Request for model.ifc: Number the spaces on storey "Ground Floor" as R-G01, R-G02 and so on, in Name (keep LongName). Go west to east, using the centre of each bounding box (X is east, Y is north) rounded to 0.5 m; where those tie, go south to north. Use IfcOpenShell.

First a look at what the model holds.

```python
import ifcopenshell
import ifcopenshell.util.element
import ifcopenshell.util.placement

model = ifcopenshell.open("model.ifc")
print(model.schema)
storey = next(s for s in model.by_type("IfcBuildingStorey") if s.Name == "Ground Floor")
spaces = [e for e in ifcopenshell.util.element.get_decomposition(storey) if e.is_a("IfcSpace")]
for e in sorted(spaces, key=lambda e: e.id()):
    origin = ifcopenshell.util.placement.get_local_placement(e.ObjectPlacement)[:3, 3]
    print(e.id(), e.Name, e.LongName, origin.round(2) + 0.0, sep=" | ")
```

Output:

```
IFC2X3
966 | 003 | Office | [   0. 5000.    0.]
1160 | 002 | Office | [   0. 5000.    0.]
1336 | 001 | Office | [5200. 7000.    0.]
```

```python
import ifcopenshell
import ifcopenshell.geom
import ifcopenshell.util.element
import ifcopenshell.util.shape

model = ifcopenshell.open("model.ifc")
settings = ifcopenshell.geom.settings()
settings.set("use-world-coords", True)


def centre(element):
    shape = ifcopenshell.geom.create_shape(settings, element)
    return ifcopenshell.util.shape.get_bbox_centroid(shape.geometry)


storey = next(s for s in model.by_type("IfcBuildingStorey") if s.Name == "Ground Floor")
spaces = [e for e in ifcopenshell.util.element.get_decomposition(storey) if e.is_a("IfcSpace")]

# Insertion points can sit at a corner or the storey origin, so sort by the geometry (in metres).
centres = {e: centre(e) for e in spaces}
spaces.sort(key=lambda e: (round(centres[e][0] / 0.5), centres[e][1]))

for i, e in enumerate(spaces, start=1):
    number = f"R-G{i:02d}"
    e.Name = number
    print(e.id(), number)

model.write("model_updated.ifc")
```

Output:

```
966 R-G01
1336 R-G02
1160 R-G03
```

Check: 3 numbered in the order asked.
